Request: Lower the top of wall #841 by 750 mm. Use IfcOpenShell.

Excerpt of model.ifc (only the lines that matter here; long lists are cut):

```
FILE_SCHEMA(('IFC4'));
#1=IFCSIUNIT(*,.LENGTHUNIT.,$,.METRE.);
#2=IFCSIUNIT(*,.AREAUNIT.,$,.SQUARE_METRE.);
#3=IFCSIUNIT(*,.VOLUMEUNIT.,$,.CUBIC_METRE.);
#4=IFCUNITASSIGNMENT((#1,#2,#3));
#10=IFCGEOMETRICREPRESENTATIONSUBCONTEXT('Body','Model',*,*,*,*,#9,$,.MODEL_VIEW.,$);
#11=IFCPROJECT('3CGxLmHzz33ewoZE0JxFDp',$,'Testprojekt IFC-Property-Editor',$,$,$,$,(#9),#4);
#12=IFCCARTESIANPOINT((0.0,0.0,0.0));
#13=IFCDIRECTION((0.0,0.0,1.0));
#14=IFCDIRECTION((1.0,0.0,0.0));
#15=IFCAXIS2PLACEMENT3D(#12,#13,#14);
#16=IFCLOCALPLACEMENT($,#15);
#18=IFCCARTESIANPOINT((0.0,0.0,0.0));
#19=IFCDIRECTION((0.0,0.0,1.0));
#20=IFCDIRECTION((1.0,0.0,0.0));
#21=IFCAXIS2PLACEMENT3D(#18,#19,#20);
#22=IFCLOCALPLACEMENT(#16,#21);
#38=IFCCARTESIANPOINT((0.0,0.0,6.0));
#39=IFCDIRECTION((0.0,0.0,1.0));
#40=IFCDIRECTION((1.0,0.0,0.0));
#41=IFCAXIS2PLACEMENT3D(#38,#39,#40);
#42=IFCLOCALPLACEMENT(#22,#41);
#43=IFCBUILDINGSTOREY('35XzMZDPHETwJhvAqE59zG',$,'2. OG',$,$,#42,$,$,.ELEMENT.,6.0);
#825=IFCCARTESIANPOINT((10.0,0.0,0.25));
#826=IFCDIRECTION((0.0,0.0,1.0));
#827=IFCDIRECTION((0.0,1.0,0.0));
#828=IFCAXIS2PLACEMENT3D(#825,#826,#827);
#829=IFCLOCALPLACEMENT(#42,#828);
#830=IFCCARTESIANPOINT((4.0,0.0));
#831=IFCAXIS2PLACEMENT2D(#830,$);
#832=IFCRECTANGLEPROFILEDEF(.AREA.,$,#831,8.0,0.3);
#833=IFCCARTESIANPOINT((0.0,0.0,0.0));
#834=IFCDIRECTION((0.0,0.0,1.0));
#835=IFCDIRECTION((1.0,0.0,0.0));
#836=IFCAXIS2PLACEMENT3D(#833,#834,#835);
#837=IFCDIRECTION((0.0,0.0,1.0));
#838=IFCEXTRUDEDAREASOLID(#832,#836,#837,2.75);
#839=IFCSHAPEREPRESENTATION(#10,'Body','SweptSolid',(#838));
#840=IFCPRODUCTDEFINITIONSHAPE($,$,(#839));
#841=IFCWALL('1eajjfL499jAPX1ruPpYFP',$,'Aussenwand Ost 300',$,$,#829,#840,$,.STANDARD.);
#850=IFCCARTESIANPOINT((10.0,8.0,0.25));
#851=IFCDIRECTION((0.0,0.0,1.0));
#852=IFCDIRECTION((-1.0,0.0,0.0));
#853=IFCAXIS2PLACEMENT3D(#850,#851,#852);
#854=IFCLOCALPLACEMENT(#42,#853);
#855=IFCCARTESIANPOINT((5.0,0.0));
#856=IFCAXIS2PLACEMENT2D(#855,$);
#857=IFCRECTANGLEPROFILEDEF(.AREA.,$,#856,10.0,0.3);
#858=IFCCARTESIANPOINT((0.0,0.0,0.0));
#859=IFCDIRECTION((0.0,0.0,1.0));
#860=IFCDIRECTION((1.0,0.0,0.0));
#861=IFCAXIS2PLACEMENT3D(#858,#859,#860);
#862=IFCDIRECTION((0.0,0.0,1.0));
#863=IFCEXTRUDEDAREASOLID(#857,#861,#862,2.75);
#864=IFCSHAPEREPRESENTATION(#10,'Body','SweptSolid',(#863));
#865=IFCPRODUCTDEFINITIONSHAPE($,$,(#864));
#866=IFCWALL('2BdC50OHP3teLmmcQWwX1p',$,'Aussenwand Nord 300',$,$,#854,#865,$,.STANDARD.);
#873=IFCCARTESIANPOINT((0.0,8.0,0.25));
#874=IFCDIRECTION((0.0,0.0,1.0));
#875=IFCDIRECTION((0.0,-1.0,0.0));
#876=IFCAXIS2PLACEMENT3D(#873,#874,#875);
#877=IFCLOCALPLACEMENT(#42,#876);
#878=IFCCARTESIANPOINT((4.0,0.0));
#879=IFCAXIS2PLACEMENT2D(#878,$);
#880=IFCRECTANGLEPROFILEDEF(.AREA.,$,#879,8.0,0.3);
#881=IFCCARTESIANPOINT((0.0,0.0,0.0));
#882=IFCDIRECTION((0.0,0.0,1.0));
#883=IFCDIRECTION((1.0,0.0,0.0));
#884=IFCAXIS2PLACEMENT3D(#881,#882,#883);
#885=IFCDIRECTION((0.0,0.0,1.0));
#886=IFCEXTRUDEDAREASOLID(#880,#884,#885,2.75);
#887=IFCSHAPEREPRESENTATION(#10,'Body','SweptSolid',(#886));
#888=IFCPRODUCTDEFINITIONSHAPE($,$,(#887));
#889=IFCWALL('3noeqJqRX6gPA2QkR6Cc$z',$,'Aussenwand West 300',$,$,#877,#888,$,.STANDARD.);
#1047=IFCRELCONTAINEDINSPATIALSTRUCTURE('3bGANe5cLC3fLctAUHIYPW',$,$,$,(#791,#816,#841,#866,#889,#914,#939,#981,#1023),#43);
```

```python
import ifcopenshell
import ifcopenshell.geom
import ifcopenshell.util.representation
import ifcopenshell.util.shape

model = ifcopenshell.open("model.ifc")
settings = ifcopenshell.geom.settings()


def volume(element):
    """Net volume in cubic metres, openings subtracted."""
    shape = ifcopenshell.geom.create_shape(settings, element)
    return ifcopenshell.util.shape.get_volume(shape.geometry)


wall = model.by_guid("1eajjfL499jAPX1ruPpYFP")
before = volume(wall)

body = ifcopenshell.util.representation.get_representation(wall, "Model", "Body")
solid = body.Items[0]
old_height = solid.Depth
solid.Depth -= 0.75
after = volume(wall)

print(f"height {old_height:g} -> {solid.Depth:g}, volume {before:.3f} -> {after:.3f} m3")

model.write("model_updated.ifc")
```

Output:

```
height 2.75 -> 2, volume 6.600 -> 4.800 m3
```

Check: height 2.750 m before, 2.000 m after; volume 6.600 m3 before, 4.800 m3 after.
